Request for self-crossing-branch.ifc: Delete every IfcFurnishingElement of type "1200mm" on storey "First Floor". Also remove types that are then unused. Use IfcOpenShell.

First a look at what the model holds.

```python
import ifcopenshell
import ifcopenshell.util.element

model = ifcopenshell.open("self-crossing-branch.ifc")
print(model.schema)
storey = next(s for s in model.by_type("IfcBuildingStorey") if s.Name == "First Floor")
furniture = [e for e in ifcopenshell.util.element.get_decomposition(storey) if e.is_a("IfcFurnishingElement")]
seen = {}
for e in furniture:
    element_type = ifcopenshell.util.element.get_type(e)
    name = element_type.Name if element_type not in (None, e) else None
    seen[name] = seen.get(name, 0) + 1
for name, count in sorted(seen.items(), key=str):
    print(count, "x", name)
```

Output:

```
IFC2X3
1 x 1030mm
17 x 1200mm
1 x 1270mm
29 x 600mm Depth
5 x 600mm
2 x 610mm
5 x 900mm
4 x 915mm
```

```python
import ifcopenshell
import ifcopenshell.api.root
import ifcopenshell.util.element

model = ifcopenshell.open("self-crossing-branch.ifc")

storey = next(s for s in model.by_type("IfcBuildingStorey") if s.Name == "First Floor")
furniture = [e for e in ifcopenshell.util.element.get_decomposition(storey) if e.is_a("IfcFurnishingElement")]
targets = [e for e in furniture if (t := ifcopenshell.util.element.get_type(e)) not in (None, e) and t.Name == "1200mm"]
types = {ifcopenshell.util.element.get_type(e) for e in targets} - {None, *targets}

for e in targets:
    ifcopenshell.api.root.remove_product(model, product=e)
print(len(targets), "removed")

unused = [t for t in types if not ifcopenshell.util.element.get_types(t)]
for t in unused:
    ifcopenshell.api.root.remove_product(model, product=t)
print(len(unused), "unused types removed")

model.write("self-crossing-branch_updated.ifc")
```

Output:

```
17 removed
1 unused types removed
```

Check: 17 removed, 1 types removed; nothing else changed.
